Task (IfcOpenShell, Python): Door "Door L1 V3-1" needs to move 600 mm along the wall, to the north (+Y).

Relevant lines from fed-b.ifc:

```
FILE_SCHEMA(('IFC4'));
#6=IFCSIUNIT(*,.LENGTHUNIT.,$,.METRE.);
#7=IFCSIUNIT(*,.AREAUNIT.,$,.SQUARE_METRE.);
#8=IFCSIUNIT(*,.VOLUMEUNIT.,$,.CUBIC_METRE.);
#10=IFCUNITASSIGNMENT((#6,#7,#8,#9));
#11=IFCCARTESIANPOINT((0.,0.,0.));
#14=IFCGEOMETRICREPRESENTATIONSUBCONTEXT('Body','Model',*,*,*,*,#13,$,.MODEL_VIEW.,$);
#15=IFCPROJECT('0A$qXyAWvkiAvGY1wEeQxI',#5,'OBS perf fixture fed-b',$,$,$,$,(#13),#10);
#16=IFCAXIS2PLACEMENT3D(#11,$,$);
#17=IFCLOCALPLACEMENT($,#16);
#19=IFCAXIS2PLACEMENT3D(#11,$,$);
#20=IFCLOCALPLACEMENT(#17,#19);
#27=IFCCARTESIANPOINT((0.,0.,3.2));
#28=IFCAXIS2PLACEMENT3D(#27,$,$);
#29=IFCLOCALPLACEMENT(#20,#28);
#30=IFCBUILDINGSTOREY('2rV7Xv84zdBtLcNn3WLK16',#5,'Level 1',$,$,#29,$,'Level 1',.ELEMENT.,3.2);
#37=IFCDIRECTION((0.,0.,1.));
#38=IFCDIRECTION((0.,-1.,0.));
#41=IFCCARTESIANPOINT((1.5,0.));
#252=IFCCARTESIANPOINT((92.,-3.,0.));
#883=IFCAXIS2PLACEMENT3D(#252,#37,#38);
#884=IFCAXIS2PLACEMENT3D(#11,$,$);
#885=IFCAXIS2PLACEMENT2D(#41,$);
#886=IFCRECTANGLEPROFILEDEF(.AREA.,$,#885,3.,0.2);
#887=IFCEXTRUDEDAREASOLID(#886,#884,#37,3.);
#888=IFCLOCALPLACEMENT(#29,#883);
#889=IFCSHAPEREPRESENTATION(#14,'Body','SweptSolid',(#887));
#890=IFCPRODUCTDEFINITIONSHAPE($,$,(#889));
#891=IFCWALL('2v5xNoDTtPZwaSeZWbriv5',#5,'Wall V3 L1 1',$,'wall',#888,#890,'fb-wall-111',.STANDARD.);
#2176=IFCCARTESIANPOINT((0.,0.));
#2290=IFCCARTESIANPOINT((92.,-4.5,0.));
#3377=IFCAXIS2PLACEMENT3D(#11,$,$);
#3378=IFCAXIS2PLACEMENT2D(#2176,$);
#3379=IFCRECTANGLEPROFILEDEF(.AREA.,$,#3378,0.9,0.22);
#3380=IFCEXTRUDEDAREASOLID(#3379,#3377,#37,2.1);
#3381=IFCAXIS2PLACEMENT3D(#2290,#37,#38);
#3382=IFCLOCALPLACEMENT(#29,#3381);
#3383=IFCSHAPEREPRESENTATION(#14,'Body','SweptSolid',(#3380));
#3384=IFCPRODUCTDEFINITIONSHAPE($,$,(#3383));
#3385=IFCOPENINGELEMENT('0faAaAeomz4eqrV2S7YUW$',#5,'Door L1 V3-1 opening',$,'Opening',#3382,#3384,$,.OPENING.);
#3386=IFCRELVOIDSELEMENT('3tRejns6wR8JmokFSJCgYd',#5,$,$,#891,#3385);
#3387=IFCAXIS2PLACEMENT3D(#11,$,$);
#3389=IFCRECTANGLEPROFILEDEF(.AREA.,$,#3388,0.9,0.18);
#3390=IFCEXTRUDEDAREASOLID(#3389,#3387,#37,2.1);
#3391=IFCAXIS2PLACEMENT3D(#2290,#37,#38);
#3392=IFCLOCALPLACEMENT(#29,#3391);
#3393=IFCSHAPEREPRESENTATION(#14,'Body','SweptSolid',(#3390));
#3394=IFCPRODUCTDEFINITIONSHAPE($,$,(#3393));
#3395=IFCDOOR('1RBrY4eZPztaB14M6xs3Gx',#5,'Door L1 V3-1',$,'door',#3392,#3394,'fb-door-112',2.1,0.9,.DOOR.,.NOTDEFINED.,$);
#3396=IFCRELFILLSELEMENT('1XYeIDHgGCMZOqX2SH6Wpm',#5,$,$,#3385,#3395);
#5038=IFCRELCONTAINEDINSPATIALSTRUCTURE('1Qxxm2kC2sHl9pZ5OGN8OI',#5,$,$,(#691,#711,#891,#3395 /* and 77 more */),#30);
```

```python
import ifcopenshell
import ifcopenshell.api.geometry
import ifcopenshell.util.placement
import ifcopenshell.util.unit

model = ifcopenshell.open("fed-b.ifc")
unit_scale = ifcopenshell.util.unit.calculate_unit_scale(model)

door = model.by_guid("1RBrY4eZPztaB14M6xs3Gx")
opening = door.FillsVoids[0].RelatingOpeningElement
wall = opening.VoidsElements[0].RelatingBuildingElement

wall_matrix = ifcopenshell.util.placement.get_local_placement(wall.ObjectPlacement)
shift = wall_matrix[:3, 0] * -0.6 / unit_scale
before = ifcopenshell.util.placement.get_local_placement(door.ObjectPlacement)[:3, 3].copy()

# The door is not placed relative to its opening, so move both.
for product in (opening, door):
    matrix = ifcopenshell.util.placement.get_local_placement(product.ObjectPlacement)
    matrix[:3, 3] += shift
    ifcopenshell.api.geometry.edit_object_placement(model, product=product, matrix=matrix, is_si=False)

after = ifcopenshell.util.placement.get_local_placement(door.ObjectPlacement)[:3, 3]
print("door moved by", (after - before).round(3) + 0.0)

model.write("fed-b_rev.ifc")
```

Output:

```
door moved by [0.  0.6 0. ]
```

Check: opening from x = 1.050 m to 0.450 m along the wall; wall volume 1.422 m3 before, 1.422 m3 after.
